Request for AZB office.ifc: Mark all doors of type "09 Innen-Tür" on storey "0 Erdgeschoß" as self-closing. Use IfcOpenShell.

First a look at what the model holds.

```python
import ifcopenshell
import ifcopenshell.util.element

model = ifcopenshell.open("AZB office.ifc")
print(model.schema)
storey = next(s for s in model.by_type("IfcBuildingStorey") if s.Name == "0 Erdgeschoß")
doors = [e for e in ifcopenshell.util.element.get_decomposition(storey) if e.is_a("IfcDoor")]
seen = {}
for e in doors:
    element_type = ifcopenshell.util.element.get_type(e)
    key = (element_type.Name if element_type != e and element_type else None, ifcopenshell.util.element.get_pset(e, "Pset_DoorCommon", "SelfClosing"))
    seen[key] = seen.get(key, 0) + 1
for (name, value), count in sorted(seen.items(), key=str):
    print(count, "x", name, "|", value)
```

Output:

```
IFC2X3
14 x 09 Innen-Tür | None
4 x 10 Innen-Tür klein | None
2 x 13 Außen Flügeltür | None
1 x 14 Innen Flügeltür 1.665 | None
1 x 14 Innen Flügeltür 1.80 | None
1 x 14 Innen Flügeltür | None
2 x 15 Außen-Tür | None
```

```python
import ifcopenshell
import ifcopenshell.api.pset
import ifcopenshell.util.element

model = ifcopenshell.open("AZB office.ifc")

storey = next(s for s in model.by_type("IfcBuildingStorey") if s.Name == "0 Erdgeschoß")
doors = [e for e in ifcopenshell.util.element.get_decomposition(storey) if e.is_a("IfcDoor")]

count = 0
for e in doors:
    element_type = ifcopenshell.util.element.get_type(e)
    if element_type in (None, e) or element_type.Name != "09 Innen-Tür":
        continue
    # add_pset returns the element's existing set when there is one.
    pset = ifcopenshell.api.pset.add_pset(model, product=e, name="Pset_DoorCommon")
    ifcopenshell.api.pset.edit_pset(model, pset=pset, properties={"SelfClosing": True})
    count += 1

print(count, "doors updated")

model.write("AZB office_rev.ifc")
```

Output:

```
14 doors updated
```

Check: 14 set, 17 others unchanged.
